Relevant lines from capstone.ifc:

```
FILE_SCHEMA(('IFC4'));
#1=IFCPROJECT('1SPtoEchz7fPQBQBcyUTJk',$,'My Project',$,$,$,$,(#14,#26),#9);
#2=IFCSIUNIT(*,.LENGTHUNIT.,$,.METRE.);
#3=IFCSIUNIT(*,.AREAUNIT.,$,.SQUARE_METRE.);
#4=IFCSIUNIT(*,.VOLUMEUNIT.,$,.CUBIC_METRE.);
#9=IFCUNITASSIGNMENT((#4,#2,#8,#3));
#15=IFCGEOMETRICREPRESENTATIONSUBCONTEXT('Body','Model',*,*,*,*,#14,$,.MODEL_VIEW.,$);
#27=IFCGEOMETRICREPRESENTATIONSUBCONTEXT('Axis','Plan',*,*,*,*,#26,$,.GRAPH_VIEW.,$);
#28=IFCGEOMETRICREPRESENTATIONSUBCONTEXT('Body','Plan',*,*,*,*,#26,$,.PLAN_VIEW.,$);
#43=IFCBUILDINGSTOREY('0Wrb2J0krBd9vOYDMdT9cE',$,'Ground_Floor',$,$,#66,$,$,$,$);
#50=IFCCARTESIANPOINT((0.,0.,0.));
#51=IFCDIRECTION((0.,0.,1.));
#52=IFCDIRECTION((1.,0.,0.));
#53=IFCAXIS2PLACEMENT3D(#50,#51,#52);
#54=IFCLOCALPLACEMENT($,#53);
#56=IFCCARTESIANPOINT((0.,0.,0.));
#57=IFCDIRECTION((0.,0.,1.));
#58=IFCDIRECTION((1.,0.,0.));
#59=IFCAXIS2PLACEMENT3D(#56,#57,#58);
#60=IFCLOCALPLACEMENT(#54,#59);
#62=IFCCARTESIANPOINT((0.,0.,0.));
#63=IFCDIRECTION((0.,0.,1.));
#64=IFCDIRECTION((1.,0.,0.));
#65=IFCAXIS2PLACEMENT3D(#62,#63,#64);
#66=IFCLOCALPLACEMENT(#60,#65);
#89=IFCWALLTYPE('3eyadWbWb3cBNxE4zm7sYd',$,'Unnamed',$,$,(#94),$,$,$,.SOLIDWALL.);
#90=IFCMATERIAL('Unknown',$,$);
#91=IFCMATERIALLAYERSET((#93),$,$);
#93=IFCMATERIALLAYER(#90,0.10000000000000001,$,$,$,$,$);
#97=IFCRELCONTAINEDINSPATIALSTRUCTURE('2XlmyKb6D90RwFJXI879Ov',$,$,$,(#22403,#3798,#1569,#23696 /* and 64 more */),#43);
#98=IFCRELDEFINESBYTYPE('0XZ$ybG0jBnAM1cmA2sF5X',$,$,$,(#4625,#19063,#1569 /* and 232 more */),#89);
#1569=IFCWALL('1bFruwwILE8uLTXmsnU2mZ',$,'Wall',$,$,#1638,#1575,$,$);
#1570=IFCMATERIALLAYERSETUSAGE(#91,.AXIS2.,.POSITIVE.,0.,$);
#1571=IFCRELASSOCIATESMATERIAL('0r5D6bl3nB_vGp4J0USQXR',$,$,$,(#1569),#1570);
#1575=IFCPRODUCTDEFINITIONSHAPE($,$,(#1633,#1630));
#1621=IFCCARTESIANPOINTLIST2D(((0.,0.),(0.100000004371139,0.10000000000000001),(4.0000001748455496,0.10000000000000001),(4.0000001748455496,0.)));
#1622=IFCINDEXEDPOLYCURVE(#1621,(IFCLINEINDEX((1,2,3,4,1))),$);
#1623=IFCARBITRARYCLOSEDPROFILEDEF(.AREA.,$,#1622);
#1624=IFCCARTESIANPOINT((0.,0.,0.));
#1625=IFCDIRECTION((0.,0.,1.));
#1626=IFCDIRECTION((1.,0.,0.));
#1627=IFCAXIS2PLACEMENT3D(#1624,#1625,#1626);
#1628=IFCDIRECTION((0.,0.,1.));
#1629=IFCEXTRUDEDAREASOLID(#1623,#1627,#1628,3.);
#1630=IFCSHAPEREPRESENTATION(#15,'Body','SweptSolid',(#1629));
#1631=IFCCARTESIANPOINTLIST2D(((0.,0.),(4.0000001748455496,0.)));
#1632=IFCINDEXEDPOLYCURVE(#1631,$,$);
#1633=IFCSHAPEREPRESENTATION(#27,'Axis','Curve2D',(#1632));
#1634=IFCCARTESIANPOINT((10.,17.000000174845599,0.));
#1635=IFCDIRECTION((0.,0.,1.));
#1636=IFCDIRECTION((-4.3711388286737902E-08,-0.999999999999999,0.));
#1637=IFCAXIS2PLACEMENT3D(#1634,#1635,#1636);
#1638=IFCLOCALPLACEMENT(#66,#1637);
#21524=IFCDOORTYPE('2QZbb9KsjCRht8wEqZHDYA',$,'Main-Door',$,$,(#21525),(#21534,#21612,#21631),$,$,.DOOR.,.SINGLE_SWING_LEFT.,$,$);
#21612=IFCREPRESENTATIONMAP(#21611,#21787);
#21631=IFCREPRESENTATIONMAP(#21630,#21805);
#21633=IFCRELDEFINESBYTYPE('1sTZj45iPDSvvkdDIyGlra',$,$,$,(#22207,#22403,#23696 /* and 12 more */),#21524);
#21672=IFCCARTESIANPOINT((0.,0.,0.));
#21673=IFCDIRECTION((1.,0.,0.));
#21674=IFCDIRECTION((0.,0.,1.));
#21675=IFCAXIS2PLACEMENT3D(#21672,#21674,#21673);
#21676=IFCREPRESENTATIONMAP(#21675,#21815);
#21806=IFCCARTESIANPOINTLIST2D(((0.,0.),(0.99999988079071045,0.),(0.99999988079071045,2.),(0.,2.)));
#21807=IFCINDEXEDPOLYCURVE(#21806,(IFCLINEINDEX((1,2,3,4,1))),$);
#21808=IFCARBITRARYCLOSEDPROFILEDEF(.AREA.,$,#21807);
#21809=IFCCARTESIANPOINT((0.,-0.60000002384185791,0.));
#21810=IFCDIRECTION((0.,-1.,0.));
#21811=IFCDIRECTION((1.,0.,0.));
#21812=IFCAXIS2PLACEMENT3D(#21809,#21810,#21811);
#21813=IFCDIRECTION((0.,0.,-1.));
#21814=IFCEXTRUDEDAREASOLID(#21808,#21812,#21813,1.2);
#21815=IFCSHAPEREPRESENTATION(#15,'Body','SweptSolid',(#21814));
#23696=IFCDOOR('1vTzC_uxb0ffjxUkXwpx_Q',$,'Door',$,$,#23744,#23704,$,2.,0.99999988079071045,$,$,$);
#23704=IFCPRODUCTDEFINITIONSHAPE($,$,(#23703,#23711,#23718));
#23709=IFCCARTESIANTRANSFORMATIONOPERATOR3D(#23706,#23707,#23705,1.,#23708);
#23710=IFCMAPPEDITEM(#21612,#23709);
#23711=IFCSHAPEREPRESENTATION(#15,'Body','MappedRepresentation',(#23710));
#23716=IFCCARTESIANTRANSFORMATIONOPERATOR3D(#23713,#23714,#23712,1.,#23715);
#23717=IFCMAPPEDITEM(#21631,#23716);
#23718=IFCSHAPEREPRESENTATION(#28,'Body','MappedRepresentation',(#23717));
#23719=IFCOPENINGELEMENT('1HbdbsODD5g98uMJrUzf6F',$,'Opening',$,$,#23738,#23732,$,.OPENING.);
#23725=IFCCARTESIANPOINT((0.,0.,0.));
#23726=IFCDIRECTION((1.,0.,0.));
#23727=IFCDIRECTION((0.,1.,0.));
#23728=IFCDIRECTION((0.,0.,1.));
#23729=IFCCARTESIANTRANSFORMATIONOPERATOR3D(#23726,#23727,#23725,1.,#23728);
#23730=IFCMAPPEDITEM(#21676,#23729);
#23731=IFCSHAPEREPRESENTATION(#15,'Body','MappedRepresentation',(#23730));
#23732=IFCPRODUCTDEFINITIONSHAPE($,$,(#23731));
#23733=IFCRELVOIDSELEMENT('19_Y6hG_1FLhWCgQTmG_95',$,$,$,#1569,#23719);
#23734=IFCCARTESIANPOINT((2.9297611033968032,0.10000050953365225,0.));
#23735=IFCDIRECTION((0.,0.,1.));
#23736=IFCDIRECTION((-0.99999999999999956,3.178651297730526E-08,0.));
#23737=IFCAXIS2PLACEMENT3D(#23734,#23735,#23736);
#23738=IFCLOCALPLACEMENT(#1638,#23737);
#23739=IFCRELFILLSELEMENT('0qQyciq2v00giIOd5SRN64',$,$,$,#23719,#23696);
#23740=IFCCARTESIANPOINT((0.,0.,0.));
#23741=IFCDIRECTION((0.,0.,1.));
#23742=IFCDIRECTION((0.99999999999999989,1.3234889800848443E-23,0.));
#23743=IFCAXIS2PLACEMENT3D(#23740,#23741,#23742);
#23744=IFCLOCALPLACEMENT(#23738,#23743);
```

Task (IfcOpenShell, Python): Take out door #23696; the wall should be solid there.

```python
import ifcopenshell
import ifcopenshell.api.feature
import ifcopenshell.api.root
import ifcopenshell.geom
import ifcopenshell.util.shape

model = ifcopenshell.open("capstone.ifc")
settings = ifcopenshell.geom.settings()


def volume(element):
    """Net volume in cubic metres, openings subtracted."""
    shape = ifcopenshell.geom.create_shape(settings, element)
    return ifcopenshell.util.shape.get_volume(shape.geometry)


door = model.by_id(23696)
opening = door.FillsVoids[0].RelatingOpeningElement
wall = opening.VoidsElements[0].RelatingBuildingElement
before = volume(wall)

ifcopenshell.api.root.remove_product(model, product=door)
ifcopenshell.api.feature.remove_feature(model, feature=opening)

after = volume(wall)

print(f"wall volume {before:.3f} -> {after:.3f} m3")

model.write("capstone-out.ifc")
```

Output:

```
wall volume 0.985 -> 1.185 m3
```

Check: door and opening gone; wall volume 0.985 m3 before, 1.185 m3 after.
